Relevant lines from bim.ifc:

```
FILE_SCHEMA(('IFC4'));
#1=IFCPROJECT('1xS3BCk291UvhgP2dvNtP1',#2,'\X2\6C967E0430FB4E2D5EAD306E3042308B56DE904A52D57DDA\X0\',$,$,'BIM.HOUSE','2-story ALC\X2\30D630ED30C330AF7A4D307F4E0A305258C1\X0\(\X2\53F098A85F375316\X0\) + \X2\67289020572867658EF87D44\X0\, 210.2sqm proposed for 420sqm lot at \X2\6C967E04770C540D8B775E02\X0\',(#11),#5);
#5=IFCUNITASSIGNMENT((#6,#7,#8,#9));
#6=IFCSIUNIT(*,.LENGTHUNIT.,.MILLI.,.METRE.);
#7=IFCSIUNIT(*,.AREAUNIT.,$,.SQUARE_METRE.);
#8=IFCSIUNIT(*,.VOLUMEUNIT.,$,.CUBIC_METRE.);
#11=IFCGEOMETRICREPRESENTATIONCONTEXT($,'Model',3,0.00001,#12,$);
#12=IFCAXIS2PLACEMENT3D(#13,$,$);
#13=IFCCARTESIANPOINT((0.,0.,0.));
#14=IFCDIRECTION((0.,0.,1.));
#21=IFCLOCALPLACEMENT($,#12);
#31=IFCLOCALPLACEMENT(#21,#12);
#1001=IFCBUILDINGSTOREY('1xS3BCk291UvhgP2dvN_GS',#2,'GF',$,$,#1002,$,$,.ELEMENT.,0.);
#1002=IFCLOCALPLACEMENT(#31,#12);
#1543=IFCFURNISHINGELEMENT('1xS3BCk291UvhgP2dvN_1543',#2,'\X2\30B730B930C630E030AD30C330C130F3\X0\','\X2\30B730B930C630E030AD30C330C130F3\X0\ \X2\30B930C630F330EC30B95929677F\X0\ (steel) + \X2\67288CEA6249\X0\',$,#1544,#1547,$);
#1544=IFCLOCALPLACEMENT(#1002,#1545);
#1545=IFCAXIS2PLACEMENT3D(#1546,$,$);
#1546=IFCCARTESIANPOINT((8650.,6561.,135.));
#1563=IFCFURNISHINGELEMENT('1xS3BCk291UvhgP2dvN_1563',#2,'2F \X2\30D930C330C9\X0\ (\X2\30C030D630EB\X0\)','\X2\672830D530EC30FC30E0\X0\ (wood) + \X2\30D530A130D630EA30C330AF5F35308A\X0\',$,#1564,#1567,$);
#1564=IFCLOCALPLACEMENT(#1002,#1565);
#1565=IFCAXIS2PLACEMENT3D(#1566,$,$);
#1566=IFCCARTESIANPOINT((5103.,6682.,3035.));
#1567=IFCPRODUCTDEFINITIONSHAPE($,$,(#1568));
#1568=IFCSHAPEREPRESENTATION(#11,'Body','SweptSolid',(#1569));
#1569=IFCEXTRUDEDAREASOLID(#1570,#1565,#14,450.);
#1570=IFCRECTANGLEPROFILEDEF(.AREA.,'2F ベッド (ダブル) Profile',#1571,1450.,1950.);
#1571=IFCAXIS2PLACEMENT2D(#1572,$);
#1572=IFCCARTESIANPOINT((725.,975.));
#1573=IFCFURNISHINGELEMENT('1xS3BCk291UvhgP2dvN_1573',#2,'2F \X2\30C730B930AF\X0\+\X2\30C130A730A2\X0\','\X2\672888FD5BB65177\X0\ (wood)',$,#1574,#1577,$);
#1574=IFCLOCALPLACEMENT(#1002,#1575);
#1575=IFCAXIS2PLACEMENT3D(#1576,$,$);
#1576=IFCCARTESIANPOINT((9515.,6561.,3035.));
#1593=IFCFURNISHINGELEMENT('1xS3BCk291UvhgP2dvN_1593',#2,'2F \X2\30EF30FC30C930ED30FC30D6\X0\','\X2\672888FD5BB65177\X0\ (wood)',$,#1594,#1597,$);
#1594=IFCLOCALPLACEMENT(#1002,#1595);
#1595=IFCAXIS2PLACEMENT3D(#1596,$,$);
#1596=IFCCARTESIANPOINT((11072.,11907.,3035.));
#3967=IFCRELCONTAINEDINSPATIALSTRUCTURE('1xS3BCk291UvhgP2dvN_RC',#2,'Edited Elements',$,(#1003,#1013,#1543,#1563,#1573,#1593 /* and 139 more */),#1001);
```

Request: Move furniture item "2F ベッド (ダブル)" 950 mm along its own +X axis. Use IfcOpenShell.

```python
import ifcopenshell
import ifcopenshell.api.geometry
import ifcopenshell.util.placement
import ifcopenshell.util.unit

model = ifcopenshell.open("bim.ifc")
unit_scale = ifcopenshell.util.unit.calculate_unit_scale(model)

item = model.by_guid("1xS3BCk291UvhgP2dvN_1563")
matrix = ifcopenshell.util.placement.get_local_placement(item.ObjectPlacement)
matrix[:3, 3] += matrix[:3, 0] * 0.95 / unit_scale
ifcopenshell.api.geometry.edit_object_placement(model, product=item, matrix=matrix, is_si=False)

print(ifcopenshell.util.placement.get_local_placement(item.ObjectPlacement).round(3) + 0.0)

model.write("bim_edited.ifc")
```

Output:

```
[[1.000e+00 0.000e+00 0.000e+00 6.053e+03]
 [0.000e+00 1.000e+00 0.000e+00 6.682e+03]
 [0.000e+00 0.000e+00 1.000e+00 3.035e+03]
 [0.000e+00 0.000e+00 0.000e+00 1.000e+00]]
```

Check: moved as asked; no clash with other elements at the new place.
